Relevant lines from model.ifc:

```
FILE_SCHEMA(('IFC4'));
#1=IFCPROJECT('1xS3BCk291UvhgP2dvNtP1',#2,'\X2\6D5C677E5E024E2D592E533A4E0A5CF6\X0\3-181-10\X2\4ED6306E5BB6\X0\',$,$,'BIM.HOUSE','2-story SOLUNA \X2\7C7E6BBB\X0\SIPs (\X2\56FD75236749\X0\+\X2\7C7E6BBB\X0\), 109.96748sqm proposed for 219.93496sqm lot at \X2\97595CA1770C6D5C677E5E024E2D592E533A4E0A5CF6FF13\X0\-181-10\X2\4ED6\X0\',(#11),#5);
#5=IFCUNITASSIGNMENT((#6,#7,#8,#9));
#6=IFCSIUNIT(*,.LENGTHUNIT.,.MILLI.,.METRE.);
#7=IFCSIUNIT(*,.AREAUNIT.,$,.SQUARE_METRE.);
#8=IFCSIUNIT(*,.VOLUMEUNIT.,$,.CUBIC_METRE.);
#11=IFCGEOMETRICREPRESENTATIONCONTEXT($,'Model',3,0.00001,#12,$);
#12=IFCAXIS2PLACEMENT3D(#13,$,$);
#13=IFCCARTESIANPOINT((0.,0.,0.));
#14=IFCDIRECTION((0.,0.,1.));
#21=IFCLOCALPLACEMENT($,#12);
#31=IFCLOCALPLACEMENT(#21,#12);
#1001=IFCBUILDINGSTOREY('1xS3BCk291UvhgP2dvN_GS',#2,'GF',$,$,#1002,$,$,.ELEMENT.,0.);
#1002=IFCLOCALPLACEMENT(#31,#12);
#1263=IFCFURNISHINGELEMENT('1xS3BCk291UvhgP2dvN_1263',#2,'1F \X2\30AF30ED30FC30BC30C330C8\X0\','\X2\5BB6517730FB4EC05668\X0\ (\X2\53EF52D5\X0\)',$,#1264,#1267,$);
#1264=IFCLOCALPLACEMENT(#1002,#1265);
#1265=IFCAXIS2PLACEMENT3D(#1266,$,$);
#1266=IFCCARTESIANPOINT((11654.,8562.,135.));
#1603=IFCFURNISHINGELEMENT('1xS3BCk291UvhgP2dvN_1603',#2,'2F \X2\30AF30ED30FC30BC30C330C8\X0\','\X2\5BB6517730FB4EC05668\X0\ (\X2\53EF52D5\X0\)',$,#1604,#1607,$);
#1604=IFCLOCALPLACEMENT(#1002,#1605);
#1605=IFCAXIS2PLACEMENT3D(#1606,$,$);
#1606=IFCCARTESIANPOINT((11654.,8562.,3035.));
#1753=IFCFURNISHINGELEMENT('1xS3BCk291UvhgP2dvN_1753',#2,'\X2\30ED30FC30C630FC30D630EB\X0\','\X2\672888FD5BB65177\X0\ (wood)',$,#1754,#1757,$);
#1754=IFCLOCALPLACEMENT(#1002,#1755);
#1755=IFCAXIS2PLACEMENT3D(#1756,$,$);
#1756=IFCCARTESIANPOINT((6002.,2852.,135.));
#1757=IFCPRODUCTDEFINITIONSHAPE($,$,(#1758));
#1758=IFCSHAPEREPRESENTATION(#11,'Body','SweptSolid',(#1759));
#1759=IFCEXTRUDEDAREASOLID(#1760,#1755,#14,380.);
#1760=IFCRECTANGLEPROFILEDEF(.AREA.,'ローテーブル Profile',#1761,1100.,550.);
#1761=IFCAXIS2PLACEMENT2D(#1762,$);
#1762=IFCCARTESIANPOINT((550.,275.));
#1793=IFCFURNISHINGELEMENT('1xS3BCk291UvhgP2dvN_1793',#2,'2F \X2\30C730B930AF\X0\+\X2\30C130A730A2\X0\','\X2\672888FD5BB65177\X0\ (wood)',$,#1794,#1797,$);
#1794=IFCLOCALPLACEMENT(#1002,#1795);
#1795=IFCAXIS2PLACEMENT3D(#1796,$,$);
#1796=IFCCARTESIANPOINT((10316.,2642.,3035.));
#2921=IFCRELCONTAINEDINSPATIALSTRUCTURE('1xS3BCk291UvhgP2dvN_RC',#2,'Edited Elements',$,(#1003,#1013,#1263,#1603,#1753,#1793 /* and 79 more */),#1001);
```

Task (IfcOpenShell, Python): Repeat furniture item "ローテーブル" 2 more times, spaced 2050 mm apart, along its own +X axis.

```python
import ifcopenshell
import ifcopenshell.api.geometry
import ifcopenshell.api.root
import ifcopenshell.util.element
import ifcopenshell.util.placement

model = ifcopenshell.open("model.ifc")


def reuse_history(source, copy):
    """copy_class also copies each property set's owner history, people and application; keep the originals."""
    for rel in copy.IsDefinedBy:
        if rel.is_a("IfcRelDefinesByProperties") and (history := rel.RelatingPropertyDefinition.OwnerHistory):
            rel.RelatingPropertyDefinition.OwnerHistory = source.OwnerHistory
            ifcopenshell.util.element.remove_deep2(model, history)


source = model.by_guid("1xS3BCk291UvhgP2dvN_1753")
base = ifcopenshell.util.placement.get_local_placement(source.ObjectPlacement)
step = base[:3, 0] * 2050.0

for i in range(1, 3):
    copy = ifcopenshell.api.root.copy_class(model, product=source)
    copy.Representation = ifcopenshell.util.element.copy_deep(
        model, source.Representation, exclude=["IfcGeometricRepresentationContext", "IfcRepresentationMap"]
    )
    reuse_history(source, copy)
    matrix = base.copy()
    matrix[:3, 3] += i * step
    print("added at", matrix[:3, 3].round(3) + 0.0)
    ifcopenshell.api.geometry.edit_object_placement(model, product=copy, matrix=matrix, is_si=False)

model.write("model-out.ifc")
```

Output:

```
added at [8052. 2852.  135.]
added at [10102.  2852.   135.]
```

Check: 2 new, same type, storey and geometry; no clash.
